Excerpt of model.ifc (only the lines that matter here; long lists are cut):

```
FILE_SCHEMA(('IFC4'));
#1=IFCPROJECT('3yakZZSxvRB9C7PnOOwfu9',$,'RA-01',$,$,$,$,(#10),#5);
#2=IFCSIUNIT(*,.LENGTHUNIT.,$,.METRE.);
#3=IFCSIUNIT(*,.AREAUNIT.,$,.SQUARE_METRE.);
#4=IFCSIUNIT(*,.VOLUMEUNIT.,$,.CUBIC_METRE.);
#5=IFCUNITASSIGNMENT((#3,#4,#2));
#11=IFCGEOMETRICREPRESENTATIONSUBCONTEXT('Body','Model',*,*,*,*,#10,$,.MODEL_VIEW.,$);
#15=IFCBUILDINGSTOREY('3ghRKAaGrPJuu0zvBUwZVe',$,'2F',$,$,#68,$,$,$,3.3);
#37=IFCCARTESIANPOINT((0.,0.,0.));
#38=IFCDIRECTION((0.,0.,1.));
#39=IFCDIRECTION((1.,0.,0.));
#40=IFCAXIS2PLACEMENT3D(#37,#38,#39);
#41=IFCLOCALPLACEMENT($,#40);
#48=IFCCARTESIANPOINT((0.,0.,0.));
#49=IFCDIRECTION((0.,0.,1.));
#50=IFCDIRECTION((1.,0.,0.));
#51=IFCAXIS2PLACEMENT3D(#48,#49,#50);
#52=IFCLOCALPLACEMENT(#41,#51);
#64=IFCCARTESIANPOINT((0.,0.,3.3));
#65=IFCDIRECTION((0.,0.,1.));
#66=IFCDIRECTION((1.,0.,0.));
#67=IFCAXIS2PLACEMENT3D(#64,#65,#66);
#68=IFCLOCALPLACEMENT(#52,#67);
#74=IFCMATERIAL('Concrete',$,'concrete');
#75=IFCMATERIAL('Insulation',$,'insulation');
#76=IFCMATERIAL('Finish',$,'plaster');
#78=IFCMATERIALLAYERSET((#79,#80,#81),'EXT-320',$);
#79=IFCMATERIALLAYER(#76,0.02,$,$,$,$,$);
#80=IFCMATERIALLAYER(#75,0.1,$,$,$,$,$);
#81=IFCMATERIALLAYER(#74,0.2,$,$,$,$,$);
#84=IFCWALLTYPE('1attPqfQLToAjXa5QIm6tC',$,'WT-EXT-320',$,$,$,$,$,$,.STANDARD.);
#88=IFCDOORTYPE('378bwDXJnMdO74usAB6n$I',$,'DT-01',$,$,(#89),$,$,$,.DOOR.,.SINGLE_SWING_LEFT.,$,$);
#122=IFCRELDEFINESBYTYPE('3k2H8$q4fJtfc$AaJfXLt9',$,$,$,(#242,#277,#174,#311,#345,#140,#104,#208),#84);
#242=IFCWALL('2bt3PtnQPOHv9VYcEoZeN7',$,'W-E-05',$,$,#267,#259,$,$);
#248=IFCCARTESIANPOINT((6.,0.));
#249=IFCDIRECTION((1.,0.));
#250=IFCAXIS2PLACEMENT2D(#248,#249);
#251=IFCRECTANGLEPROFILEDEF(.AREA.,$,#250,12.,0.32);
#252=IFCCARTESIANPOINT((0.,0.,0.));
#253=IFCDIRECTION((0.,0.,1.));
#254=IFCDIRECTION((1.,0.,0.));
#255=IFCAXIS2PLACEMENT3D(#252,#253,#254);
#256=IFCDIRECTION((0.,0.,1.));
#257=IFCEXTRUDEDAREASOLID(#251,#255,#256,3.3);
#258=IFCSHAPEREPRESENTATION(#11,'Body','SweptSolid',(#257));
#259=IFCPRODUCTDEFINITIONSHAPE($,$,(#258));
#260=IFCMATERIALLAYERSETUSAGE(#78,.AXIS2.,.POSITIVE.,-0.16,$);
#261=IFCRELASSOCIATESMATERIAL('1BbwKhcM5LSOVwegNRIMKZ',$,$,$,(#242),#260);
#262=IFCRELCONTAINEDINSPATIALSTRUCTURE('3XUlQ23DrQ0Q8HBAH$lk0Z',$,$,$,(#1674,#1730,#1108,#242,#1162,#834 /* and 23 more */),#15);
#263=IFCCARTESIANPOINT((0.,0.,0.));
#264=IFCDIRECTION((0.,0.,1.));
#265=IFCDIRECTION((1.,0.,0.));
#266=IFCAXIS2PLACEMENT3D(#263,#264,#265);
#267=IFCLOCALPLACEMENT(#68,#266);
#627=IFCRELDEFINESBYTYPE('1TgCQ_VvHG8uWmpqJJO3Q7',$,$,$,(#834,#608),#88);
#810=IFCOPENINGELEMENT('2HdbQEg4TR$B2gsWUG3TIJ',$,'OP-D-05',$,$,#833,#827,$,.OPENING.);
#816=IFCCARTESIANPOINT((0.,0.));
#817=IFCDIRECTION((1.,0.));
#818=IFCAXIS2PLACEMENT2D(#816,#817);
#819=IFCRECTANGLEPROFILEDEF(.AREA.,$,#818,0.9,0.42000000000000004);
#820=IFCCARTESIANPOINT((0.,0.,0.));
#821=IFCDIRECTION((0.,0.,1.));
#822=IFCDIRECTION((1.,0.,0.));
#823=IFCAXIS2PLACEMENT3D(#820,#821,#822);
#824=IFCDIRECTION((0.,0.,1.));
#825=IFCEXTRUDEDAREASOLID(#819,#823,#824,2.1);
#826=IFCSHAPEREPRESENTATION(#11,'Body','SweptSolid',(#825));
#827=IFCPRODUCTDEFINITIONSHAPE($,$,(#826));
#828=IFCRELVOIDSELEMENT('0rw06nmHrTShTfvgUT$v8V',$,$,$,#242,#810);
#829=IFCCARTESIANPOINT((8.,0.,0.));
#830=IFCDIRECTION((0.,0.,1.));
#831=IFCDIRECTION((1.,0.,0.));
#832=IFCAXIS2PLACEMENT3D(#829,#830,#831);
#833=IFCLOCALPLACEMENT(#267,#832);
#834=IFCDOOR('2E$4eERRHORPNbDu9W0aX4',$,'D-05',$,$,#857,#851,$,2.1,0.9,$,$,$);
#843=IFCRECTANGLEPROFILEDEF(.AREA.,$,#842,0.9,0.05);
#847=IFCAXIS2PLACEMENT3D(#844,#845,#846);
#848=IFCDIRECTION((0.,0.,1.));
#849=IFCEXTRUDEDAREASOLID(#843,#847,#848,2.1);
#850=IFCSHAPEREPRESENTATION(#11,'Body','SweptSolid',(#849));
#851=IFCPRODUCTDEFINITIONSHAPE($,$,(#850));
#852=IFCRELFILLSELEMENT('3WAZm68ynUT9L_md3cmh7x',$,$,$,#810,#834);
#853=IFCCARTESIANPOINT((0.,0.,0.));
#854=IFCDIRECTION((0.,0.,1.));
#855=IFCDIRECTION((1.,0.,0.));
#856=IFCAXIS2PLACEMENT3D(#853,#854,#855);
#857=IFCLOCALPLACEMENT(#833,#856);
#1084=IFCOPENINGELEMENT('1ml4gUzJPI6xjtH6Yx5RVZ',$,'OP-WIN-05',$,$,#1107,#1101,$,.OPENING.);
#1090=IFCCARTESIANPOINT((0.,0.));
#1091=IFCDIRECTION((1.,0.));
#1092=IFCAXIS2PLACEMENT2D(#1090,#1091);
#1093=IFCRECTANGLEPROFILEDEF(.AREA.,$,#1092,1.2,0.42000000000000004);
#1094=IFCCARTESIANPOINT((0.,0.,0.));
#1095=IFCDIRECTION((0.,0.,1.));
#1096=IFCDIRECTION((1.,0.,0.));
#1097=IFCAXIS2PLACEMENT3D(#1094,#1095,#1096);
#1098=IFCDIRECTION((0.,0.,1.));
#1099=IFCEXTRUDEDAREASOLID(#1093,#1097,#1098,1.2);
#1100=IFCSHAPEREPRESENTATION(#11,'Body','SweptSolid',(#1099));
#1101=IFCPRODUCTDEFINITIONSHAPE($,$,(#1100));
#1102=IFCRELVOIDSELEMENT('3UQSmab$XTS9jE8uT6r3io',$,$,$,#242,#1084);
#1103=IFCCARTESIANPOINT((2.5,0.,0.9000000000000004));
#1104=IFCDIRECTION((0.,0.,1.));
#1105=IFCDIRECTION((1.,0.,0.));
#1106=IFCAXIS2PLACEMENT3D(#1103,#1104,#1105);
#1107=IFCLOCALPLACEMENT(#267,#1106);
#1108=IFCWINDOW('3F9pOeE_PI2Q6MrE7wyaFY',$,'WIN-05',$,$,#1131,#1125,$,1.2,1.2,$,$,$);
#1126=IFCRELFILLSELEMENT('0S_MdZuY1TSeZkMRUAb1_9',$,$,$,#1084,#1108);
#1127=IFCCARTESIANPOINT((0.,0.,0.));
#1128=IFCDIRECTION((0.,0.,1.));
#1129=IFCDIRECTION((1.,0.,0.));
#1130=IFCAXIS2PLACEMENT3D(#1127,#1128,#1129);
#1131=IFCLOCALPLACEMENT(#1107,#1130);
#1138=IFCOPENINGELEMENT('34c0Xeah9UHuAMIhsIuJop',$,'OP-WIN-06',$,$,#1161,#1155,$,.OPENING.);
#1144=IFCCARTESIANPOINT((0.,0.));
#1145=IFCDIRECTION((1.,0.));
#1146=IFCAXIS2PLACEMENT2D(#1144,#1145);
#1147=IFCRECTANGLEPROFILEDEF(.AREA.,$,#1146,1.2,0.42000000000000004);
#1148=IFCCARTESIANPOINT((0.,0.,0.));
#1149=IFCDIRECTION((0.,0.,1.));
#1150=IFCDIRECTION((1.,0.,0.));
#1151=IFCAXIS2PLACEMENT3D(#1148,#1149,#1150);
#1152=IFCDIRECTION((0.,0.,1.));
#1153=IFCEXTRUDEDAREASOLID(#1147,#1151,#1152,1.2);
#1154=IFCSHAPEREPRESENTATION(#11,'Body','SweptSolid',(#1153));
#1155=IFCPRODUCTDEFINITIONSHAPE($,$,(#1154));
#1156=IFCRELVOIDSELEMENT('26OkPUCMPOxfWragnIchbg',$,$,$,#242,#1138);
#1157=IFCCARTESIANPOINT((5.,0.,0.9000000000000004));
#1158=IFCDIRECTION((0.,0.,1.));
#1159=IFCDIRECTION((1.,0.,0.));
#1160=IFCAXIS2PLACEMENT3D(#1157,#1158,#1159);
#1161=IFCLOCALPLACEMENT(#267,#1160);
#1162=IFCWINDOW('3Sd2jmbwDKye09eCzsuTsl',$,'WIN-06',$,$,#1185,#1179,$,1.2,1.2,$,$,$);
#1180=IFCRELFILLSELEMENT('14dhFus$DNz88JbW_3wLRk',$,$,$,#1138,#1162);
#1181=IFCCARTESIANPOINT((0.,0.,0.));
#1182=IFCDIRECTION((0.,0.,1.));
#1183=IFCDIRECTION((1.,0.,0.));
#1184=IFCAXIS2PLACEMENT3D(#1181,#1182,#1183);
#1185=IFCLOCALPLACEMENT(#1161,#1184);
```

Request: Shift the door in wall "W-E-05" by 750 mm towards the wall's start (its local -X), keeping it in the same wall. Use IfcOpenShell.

```python
import ifcopenshell
import ifcopenshell.api.geometry
import ifcopenshell.util.placement
import ifcopenshell.util.unit

model = ifcopenshell.open("model.ifc")
unit_scale = ifcopenshell.util.unit.calculate_unit_scale(model)

door = model.by_guid("2E$4eERRHORPNbDu9W0aX4")
opening = door.FillsVoids[0].RelatingOpeningElement
wall = opening.VoidsElements[0].RelatingBuildingElement

wall_matrix = ifcopenshell.util.placement.get_local_placement(wall.ObjectPlacement)
shift = wall_matrix[:3, 0] * -0.75 / unit_scale
before = ifcopenshell.util.placement.get_local_placement(door.ObjectPlacement)[:3, 3].copy()

# The door is placed relative to its opening, so it follows when the opening moves.
matrix = ifcopenshell.util.placement.get_local_placement(opening.ObjectPlacement)
matrix[:3, 3] += shift
ifcopenshell.api.geometry.edit_object_placement(
    model, product=opening, matrix=matrix, is_si=False, should_transform_children=True
)

after = ifcopenshell.util.placement.get_local_placement(door.ObjectPlacement)[:3, 3]
print("door moved by", (after - before).round(3) + 0.0)

model.write("model_edited.ifc")
```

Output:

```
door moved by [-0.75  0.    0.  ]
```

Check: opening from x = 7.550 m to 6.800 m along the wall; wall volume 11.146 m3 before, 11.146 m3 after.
